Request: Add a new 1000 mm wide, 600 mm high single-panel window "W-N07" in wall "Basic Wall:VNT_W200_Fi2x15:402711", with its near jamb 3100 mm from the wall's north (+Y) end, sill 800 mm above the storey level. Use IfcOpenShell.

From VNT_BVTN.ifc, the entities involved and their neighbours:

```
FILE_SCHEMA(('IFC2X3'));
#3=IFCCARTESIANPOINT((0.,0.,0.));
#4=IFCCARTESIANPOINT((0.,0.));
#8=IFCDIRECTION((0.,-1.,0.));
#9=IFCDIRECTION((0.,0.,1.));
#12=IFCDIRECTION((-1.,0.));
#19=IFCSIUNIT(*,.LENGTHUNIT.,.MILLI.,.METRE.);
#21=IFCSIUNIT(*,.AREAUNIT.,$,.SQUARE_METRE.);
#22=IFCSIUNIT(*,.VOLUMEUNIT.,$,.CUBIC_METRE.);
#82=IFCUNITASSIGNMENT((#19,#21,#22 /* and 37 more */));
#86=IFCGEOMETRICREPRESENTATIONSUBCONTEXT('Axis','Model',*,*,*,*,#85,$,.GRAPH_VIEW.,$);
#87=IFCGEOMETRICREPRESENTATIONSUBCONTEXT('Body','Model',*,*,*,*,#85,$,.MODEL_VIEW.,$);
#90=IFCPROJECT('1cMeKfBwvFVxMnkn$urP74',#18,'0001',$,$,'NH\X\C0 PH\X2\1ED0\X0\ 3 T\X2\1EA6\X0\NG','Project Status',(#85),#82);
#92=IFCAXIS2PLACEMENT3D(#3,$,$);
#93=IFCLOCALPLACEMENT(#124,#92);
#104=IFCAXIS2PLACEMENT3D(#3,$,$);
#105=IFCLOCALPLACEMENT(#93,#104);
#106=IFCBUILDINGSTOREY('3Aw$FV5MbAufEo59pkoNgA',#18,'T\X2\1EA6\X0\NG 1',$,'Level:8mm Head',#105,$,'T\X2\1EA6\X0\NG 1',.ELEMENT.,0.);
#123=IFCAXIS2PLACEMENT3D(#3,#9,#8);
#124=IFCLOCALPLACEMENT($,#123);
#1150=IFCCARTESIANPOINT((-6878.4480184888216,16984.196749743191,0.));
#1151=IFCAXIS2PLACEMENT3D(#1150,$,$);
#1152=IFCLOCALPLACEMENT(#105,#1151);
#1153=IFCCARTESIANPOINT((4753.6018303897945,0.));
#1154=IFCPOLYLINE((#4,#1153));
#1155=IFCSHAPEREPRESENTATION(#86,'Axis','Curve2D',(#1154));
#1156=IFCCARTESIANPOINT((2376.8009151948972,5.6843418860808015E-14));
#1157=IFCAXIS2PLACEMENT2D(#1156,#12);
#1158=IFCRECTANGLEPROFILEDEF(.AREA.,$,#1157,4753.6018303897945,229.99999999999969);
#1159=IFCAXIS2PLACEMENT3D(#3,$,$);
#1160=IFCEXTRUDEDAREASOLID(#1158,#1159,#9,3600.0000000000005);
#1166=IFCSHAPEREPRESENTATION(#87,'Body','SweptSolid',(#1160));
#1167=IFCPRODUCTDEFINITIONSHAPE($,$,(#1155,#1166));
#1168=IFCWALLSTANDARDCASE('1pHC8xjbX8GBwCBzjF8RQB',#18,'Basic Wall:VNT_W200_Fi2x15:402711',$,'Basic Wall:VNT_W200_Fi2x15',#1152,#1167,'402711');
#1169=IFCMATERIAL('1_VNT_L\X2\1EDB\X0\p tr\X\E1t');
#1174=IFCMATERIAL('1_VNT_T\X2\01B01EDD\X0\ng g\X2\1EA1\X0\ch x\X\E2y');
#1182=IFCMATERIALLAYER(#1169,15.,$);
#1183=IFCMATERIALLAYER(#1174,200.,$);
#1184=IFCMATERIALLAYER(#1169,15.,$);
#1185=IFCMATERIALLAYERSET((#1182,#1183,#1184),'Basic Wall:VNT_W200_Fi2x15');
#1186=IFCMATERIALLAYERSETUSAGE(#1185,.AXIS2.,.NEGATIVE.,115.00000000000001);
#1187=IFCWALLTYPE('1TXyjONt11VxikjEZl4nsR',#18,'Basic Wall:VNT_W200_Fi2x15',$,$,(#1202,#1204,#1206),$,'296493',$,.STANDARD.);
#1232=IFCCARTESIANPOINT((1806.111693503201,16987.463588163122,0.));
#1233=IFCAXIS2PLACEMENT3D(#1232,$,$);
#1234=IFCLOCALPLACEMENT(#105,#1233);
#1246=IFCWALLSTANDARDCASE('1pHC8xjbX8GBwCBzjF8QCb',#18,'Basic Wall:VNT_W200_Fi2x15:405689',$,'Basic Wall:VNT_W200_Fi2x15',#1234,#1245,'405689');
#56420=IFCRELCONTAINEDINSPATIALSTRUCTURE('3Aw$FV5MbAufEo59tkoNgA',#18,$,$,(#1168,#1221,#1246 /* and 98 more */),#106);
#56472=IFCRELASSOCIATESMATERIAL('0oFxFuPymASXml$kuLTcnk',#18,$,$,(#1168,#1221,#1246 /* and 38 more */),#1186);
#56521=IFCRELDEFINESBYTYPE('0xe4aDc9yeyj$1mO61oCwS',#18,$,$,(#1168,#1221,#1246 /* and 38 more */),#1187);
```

```python
import numpy as np
import ifcopenshell
import ifcopenshell.api.feature
import ifcopenshell.api.geometry
import ifcopenshell.api.root
import ifcopenshell.api.spatial
import ifcopenshell.api.type
import ifcopenshell.geom
import ifcopenshell.util.element
import ifcopenshell.util.placement
import ifcopenshell.util.representation
import ifcopenshell.util.shape
import ifcopenshell.util.unit

model = ifcopenshell.open("VNT_BVTN.ifc")
unit_scale = ifcopenshell.util.unit.calculate_unit_scale(model)
settings = ifcopenshell.geom.settings()


def volume(element):
    """Net volume in cubic metres, openings subtracted."""
    shape = ifcopenshell.geom.create_shape(settings, element)
    return ifcopenshell.util.shape.get_volume(shape.geometry)


wall = model.by_guid("1pHC8xjbX8GBwCBzjF8RQB")
storey = ifcopenshell.util.element.get_container(wall, ifc_class="IfcBuildingStorey")
context = ifcopenshell.util.representation.get_context(model, "Model", "Body", "MODEL_VIEW")
before = volume(wall)

width, height, from_end, sill = 1, 0.6, 3.1, 0.8  # metres

# The wall runs along its own X axis, and the end named is its -X end.
wall_shape = ifcopenshell.geom.create_shape(settings, wall)
x, y, z = ifcopenshell.util.shape.get_vertices(wall_shape.geometry).T
start = x.min() + from_end
face, thickness = float(y.min()), float(y.max() - y.min())
wall_matrix = ifcopenshell.util.placement.get_local_placement(wall.ObjectPlacement)
level = ifcopenshell.util.placement.get_local_placement(storey.ObjectPlacement)[2, 3]


def in_wall(x, y):
    """Placement at x, y metres in the wall's axes, at sill height."""
    matrix = wall_matrix.copy()
    matrix[:, 3] = wall_matrix @ np.array([x / unit_scale, y / unit_scale, 0.0, 1.0])
    matrix[2, 3] = level + sill / unit_scale
    return matrix


# Opening: a box that overshoots both wall faces by 50 mm.
opening = ifcopenshell.api.root.create_entity(model, ifc_class="IfcOpeningElement")
box = ifcopenshell.api.geometry.add_wall_representation(
    model, context=context, length=width, height=height, thickness=thickness + 0.1
)
ifcopenshell.api.geometry.assign_representation(model, product=opening, representation=box)
ifcopenshell.api.geometry.edit_object_placement(model, product=opening, matrix=in_wall(start, face - 0.05), is_si=False)
ifcopenshell.api.feature.add_feature(model, feature=opening, element=wall)

window = ifcopenshell.api.root.create_entity(model, ifc_class="IfcWindow", name="W-N07")
window.OverallWidth, window.OverallHeight = width / unit_scale, height / unit_scale
body = ifcopenshell.api.geometry.add_window_representation(
    model,
    context=context,
    overall_width=window.OverallWidth,
    overall_height=window.OverallHeight,
    partition_type="SINGLE_PANEL",
)
ifcopenshell.api.geometry.assign_representation(model, product=window, representation=body)
ifcopenshell.api.spatial.assign_container(model, products=[window], relating_structure=storey)
fills = ifcopenshell.api.feature.add_filling(model, opening=opening, element=window)
fills.OwnerHistory = window.OwnerHistory  # required in IFC2X3

# IFC2X3 keeps the operation on the window style.
style = ifcopenshell.api.root.create_entity(model, ifc_class="IfcWindowStyle", name="W-N07")
style.OperationType, style.ConstructionType = "SINGLE_PANEL", "NOTDEFINED"
style.ParameterTakesPrecedence = style.Sizeable = False
ifcopenshell.api.type.assign_type(model, related_objects=[window], relating_type=style)

# Centre the window in the wall's thickness.
ifcopenshell.api.geometry.edit_object_placement(model, product=window, matrix=in_wall(start, face), is_si=False)
window_shape = ifcopenshell.geom.create_shape(settings, window)
depth = ifcopenshell.util.shape.get_vertices(window_shape.geometry)[:, 1]
offset = face + thickness / 2 - (depth.min() + depth.max()) / 2
ifcopenshell.api.geometry.edit_object_placement(model, product=window, matrix=in_wall(start, offset), is_si=False)

after = volume(wall)

print(f"wall volume {before:.3f} -> {after:.3f} m3")

model.write("VNT_BVTN_updated.ifc")
```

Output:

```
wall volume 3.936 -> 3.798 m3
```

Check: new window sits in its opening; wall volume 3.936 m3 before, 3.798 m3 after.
